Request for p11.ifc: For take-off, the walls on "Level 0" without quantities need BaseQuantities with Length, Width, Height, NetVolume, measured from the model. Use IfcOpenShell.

First a look at what the model holds.

```python
import ifcopenshell
import ifcopenshell.util.element
import ifcopenshell.util.unit

model = ifcopenshell.open("p11.ifc")
print(model.schema)
for unit_type in ("LENGTHUNIT", "AREAUNIT", "VOLUMEUNIT"):
    print(unit_type, ifcopenshell.util.unit.calculate_unit_scale(model, unit_type))
storey = next(s for s in model.by_type("IfcBuildingStorey") if s.Name == "Level 0")
walls = [e for e in ifcopenshell.util.element.get_decomposition(storey) if e.is_a("IfcWall")]
for e in sorted(walls, key=lambda e: e.id()):
    print(e.id(), e.is_a(), e.Name, list(ifcopenshell.util.element.get_psets(e, qtos_only=True)), sep=" | ")
```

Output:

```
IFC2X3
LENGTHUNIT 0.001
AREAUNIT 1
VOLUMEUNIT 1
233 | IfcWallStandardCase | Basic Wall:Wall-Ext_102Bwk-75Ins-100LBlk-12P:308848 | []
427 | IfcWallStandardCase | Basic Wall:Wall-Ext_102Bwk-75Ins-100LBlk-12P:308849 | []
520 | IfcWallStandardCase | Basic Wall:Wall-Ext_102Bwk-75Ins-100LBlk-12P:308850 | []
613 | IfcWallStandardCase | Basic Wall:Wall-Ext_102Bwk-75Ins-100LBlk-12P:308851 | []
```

```python
import ifcopenshell
import ifcopenshell.api.pset
import ifcopenshell.geom
import ifcopenshell.util.element
import ifcopenshell.util.shape
import ifcopenshell.util.unit

model = ifcopenshell.open("p11.ifc")
unit_scale = ifcopenshell.util.unit.calculate_unit_scale(model)
volume_scale = ifcopenshell.util.unit.calculate_unit_scale(model, "VOLUMEUNIT")
settings = ifcopenshell.geom.settings()

storey = next(s for s in model.by_type("IfcBuildingStorey") if s.Name == "Level 0")
walls = [e for e in ifcopenshell.util.element.get_decomposition(storey) if e.is_a("IfcWall")]

for e in sorted(walls, key=lambda e: e.id()):
    if ifcopenshell.util.element.get_psets(e, qtos_only=True, should_inherit=False):
        continue
    # Geometry comes back in metres, in the element's own axes.
    shape = ifcopenshell.geom.create_shape(settings, e)
    values = {
        "Length": ifcopenshell.util.shape.get_x(shape.geometry) / unit_scale,
        "Width": ifcopenshell.util.shape.get_y(shape.geometry) / unit_scale,
        "Height": ifcopenshell.util.shape.get_z(shape.geometry) / unit_scale,
        "NetVolume": ifcopenshell.util.shape.get_volume(shape.geometry) / volume_scale,
    }
    qto = ifcopenshell.api.pset.add_qto(model, product=e, name="BaseQuantities")
    ifcopenshell.api.pset.edit_qto(model, qto=qto, properties=values)
    print(e.id(), {k: round(v, 3) for k, v in values.items()})

model.write("p11_updated.ifc")
```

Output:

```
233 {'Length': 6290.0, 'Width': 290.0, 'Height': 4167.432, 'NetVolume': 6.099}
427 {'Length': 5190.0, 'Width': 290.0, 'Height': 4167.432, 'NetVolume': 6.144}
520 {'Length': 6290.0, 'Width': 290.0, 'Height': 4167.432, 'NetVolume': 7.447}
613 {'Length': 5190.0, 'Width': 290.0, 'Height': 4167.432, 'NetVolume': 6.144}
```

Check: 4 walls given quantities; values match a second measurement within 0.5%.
